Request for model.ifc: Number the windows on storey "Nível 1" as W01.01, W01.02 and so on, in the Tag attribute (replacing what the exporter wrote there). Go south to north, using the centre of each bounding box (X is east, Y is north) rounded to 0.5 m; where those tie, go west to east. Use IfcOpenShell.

First a look at what the model holds.

```python
import ifcopenshell
import ifcopenshell.util.element
import ifcopenshell.util.placement

model = ifcopenshell.open("model.ifc")
print(model.schema)
storey = next(s for s in model.by_type("IfcBuildingStorey") if s.Name == "Nível 1")
windows = [e for e in ifcopenshell.util.element.get_decomposition(storey) if e.is_a("IfcWindow")]
for e in sorted(windows, key=lambda e: e.id()):
    origin = ifcopenshell.util.placement.get_local_placement(e.ObjectPlacement)[:3, 3]
    print(e.id(), e.Tag, e.Name, origin.round(2) + 0.0, sep=" | ")
```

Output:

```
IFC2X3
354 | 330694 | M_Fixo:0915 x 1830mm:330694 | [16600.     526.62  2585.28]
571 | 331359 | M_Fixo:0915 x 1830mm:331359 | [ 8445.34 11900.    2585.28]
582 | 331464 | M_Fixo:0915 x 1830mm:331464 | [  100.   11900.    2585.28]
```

```python
import ifcopenshell
import ifcopenshell.geom
import ifcopenshell.util.element
import ifcopenshell.util.shape

model = ifcopenshell.open("model.ifc")
settings = ifcopenshell.geom.settings()
settings.set("use-world-coords", True)


def centre(element):
    shape = ifcopenshell.geom.create_shape(settings, element)
    return ifcopenshell.util.shape.get_bbox_centroid(shape.geometry)


storey = next(s for s in model.by_type("IfcBuildingStorey") if s.Name == "Nível 1")
windows = [e for e in ifcopenshell.util.element.get_decomposition(storey) if e.is_a("IfcWindow")]

# Insertion points can sit at a corner or the storey origin, so sort by the geometry (in metres).
centres = {e: centre(e) for e in windows}
windows.sort(key=lambda e: (round(centres[e][1] / 0.5), centres[e][0]))

for i, e in enumerate(windows, start=1):
    number = f"W01.{i:02d}"
    e.Tag = number
    print(e.id(), number)

model.write("model_edited.ifc")
```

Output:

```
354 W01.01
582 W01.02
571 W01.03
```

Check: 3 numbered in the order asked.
